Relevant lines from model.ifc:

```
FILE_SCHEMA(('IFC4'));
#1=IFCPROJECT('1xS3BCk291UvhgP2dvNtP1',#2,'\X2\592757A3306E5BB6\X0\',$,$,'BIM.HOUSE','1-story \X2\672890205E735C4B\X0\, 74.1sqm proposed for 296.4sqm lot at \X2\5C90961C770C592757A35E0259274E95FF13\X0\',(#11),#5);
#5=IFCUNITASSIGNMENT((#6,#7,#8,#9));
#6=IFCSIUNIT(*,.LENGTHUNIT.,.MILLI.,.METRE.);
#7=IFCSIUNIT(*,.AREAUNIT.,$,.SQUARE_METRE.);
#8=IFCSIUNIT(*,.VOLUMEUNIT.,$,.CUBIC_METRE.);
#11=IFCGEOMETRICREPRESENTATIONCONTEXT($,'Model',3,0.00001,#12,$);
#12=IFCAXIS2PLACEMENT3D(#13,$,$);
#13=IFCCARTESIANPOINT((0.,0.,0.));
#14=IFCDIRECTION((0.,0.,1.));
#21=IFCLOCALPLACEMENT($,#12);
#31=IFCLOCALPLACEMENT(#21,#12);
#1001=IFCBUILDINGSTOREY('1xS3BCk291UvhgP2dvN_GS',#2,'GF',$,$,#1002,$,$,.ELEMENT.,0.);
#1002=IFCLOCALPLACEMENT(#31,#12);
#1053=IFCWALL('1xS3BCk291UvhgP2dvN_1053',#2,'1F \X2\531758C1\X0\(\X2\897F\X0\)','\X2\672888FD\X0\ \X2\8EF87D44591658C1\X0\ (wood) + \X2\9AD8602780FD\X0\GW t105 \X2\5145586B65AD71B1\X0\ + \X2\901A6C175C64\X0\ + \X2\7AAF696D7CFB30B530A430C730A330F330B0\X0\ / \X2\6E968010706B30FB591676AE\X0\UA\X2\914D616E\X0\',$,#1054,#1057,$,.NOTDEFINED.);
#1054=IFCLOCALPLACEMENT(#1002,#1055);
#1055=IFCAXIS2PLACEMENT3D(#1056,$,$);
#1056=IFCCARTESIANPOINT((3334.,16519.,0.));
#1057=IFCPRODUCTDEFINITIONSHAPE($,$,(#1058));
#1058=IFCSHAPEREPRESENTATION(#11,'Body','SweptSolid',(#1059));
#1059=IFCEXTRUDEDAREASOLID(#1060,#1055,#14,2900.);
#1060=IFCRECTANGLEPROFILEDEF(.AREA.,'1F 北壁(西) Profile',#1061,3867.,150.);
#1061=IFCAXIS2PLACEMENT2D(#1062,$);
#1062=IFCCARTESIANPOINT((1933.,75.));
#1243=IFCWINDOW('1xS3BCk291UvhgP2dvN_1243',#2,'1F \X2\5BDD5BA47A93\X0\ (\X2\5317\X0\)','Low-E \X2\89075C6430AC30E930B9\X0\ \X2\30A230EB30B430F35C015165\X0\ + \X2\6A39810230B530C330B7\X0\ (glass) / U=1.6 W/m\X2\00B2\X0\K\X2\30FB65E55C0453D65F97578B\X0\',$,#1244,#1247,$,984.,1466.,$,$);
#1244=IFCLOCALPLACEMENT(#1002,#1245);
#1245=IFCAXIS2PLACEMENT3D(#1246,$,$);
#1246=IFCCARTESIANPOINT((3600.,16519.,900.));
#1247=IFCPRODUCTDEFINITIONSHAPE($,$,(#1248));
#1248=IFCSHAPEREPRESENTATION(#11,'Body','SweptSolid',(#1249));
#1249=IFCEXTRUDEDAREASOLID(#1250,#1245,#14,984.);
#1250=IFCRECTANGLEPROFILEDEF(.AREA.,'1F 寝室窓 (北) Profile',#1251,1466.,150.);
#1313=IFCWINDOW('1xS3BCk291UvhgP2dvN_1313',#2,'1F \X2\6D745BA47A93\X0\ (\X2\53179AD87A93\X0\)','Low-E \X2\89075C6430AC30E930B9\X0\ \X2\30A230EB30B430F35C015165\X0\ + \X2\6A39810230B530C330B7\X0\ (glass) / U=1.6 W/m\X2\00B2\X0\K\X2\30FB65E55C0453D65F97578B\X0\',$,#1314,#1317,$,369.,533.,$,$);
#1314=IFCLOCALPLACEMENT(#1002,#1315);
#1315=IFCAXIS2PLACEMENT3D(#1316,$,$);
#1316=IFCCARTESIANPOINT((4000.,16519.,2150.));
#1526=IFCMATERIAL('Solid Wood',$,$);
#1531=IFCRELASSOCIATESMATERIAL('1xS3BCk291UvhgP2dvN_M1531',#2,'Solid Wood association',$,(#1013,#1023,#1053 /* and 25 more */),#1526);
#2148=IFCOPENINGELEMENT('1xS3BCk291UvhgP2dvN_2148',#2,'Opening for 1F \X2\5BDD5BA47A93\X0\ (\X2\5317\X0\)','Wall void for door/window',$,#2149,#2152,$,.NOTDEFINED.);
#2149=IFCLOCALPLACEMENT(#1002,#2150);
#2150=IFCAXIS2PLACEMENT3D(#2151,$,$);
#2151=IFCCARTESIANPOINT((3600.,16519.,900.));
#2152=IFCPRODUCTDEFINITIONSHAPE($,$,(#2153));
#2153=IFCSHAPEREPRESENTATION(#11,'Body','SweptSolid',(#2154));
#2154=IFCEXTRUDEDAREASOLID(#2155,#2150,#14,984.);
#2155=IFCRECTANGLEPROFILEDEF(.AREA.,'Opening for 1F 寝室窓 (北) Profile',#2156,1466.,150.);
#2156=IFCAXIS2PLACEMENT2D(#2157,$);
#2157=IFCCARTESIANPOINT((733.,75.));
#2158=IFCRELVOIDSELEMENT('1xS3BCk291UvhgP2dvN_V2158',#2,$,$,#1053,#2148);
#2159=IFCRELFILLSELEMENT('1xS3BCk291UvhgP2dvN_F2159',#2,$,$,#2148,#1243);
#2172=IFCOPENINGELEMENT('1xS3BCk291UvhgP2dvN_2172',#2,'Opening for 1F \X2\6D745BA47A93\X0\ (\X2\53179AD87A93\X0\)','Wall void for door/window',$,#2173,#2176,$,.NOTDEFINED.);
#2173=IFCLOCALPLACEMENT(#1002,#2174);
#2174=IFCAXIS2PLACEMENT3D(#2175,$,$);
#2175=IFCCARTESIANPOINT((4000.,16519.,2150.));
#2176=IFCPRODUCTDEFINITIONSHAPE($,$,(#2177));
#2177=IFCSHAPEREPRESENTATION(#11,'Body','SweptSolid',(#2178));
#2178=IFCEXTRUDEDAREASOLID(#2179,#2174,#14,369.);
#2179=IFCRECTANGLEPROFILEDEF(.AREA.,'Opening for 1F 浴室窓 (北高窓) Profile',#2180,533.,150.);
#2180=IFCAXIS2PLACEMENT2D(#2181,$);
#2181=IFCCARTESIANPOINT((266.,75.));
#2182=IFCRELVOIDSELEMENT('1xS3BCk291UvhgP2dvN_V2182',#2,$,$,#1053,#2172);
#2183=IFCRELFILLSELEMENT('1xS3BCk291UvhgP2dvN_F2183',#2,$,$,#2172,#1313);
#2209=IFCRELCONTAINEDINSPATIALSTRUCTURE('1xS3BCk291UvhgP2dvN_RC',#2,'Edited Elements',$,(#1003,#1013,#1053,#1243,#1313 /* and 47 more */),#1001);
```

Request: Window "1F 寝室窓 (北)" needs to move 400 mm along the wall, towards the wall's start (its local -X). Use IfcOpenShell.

```python
import ifcopenshell
import ifcopenshell.api.geometry
import ifcopenshell.util.placement
import ifcopenshell.util.unit

model = ifcopenshell.open("model.ifc")
unit_scale = ifcopenshell.util.unit.calculate_unit_scale(model)

window = model.by_guid("1xS3BCk291UvhgP2dvN_1243")
opening = window.FillsVoids[0].RelatingOpeningElement
wall = opening.VoidsElements[0].RelatingBuildingElement

wall_matrix = ifcopenshell.util.placement.get_local_placement(wall.ObjectPlacement)
shift = wall_matrix[:3, 0] * -0.4 / unit_scale
before = ifcopenshell.util.placement.get_local_placement(window.ObjectPlacement)[:3, 3].copy()

# The window is not placed relative to its opening, so move both.
for product in (opening, window):
    matrix = ifcopenshell.util.placement.get_local_placement(product.ObjectPlacement)
    matrix[:3, 3] += shift
    ifcopenshell.api.geometry.edit_object_placement(model, product=product, matrix=matrix, is_si=False)

after = ifcopenshell.util.placement.get_local_placement(window.ObjectPlacement)[:3, 3]
print("window moved by", (after - before).round(3) + 0.0)

model.write("model_rev.ifc")
```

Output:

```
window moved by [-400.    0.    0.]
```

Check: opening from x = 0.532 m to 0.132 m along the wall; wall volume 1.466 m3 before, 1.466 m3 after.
